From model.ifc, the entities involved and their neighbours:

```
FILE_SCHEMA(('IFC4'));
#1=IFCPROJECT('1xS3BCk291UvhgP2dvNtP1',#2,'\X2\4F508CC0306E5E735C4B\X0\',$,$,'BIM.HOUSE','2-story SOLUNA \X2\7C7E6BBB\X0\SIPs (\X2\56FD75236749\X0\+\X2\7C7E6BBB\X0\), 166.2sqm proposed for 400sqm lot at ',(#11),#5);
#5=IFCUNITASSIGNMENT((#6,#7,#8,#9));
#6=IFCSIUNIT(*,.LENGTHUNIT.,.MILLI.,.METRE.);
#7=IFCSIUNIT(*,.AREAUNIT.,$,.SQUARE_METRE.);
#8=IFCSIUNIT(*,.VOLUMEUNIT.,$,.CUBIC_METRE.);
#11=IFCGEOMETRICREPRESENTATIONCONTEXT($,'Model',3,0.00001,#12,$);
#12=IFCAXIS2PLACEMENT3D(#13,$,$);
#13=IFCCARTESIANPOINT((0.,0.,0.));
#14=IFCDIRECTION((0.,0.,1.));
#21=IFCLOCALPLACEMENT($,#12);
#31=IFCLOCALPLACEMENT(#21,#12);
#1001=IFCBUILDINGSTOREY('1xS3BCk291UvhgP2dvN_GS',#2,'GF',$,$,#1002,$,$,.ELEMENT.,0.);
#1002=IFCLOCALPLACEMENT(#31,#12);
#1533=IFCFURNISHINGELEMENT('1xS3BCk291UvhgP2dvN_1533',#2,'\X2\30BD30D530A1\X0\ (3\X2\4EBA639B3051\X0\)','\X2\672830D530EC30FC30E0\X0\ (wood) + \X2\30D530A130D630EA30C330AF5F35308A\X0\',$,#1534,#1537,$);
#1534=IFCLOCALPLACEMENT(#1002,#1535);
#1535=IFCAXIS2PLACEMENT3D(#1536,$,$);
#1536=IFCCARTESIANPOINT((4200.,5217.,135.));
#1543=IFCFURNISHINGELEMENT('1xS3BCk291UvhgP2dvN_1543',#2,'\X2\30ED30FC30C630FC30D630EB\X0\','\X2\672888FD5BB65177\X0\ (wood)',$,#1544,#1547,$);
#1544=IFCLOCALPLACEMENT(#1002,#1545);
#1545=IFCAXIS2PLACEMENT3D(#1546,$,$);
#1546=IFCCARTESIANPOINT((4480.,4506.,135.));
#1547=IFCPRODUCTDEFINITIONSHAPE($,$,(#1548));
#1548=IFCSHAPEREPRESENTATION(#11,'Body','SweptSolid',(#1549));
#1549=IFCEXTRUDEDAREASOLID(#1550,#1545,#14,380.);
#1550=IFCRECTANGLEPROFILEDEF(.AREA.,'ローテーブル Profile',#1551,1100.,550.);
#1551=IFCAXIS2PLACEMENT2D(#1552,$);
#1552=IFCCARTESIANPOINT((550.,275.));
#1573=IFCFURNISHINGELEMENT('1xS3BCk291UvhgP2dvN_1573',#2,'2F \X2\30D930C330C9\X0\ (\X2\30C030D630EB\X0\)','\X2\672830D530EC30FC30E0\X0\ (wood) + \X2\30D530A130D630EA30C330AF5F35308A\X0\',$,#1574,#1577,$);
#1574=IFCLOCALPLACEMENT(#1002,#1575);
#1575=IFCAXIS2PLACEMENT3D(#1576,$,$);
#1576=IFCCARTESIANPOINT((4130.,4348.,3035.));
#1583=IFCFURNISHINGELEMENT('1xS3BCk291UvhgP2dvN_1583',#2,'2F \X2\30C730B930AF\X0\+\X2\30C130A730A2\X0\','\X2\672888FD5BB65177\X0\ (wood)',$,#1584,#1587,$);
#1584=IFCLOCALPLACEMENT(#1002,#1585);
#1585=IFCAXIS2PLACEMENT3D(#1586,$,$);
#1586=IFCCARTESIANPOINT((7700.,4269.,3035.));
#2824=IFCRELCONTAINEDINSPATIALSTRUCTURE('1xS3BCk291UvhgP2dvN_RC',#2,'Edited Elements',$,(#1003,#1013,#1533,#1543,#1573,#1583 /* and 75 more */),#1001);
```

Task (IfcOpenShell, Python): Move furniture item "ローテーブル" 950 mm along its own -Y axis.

```python
import ifcopenshell
import ifcopenshell.api.geometry
import ifcopenshell.util.placement

model = ifcopenshell.open("model.ifc")

item = model.by_id(1543)
matrix = ifcopenshell.util.placement.get_local_placement(item.ObjectPlacement)
matrix[:3, 3] -= matrix[:3, 1] * 950.0
ifcopenshell.api.geometry.edit_object_placement(model, product=item, matrix=matrix, is_si=False)

print(ifcopenshell.util.placement.get_local_placement(item.ObjectPlacement).round(3) + 0.0)

model.write("model_updated.ifc")
```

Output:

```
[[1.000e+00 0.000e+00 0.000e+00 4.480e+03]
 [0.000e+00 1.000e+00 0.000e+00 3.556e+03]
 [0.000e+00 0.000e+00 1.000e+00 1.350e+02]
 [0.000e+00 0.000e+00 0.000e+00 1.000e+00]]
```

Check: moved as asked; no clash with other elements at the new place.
